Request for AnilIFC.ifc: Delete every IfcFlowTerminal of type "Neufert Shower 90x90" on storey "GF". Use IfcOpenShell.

First a look at what the model holds.

```python
import ifcopenshell
import ifcopenshell.util.element

model = ifcopenshell.open("AnilIFC.ifc")
print(model.schema)
storey = next(s for s in model.by_type("IfcBuildingStorey") if s.Name == "GF")
terminals = [e for e in ifcopenshell.util.element.get_decomposition(storey) if e.is_a("IfcFlowTerminal")]
seen = {}
for e in terminals:
    element_type = ifcopenshell.util.element.get_type(e)
    name = element_type.Name if element_type not in (None, e) else None
    seen[name] = seen.get(name, 0) + 1
for name, count in sorted(seen.items(), key=str):
    print(count, "x", name)
```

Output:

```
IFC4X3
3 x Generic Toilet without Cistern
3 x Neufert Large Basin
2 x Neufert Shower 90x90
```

```python
import ifcopenshell
import ifcopenshell.api.root
import ifcopenshell.util.element

model = ifcopenshell.open("AnilIFC.ifc")

storey = next(s for s in model.by_type("IfcBuildingStorey") if s.Name == "GF")
terminals = [e for e in ifcopenshell.util.element.get_decomposition(storey) if e.is_a("IfcFlowTerminal")]
targets = [e for e in terminals if (t := ifcopenshell.util.element.get_type(e)) not in (None, e) and t.Name == "Neufert Shower 90x90"]

for e in targets:
    ifcopenshell.api.root.remove_product(model, product=e)
print(len(targets), "removed")

model.write("AnilIFC_edited.ifc")
```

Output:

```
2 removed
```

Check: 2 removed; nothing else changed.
